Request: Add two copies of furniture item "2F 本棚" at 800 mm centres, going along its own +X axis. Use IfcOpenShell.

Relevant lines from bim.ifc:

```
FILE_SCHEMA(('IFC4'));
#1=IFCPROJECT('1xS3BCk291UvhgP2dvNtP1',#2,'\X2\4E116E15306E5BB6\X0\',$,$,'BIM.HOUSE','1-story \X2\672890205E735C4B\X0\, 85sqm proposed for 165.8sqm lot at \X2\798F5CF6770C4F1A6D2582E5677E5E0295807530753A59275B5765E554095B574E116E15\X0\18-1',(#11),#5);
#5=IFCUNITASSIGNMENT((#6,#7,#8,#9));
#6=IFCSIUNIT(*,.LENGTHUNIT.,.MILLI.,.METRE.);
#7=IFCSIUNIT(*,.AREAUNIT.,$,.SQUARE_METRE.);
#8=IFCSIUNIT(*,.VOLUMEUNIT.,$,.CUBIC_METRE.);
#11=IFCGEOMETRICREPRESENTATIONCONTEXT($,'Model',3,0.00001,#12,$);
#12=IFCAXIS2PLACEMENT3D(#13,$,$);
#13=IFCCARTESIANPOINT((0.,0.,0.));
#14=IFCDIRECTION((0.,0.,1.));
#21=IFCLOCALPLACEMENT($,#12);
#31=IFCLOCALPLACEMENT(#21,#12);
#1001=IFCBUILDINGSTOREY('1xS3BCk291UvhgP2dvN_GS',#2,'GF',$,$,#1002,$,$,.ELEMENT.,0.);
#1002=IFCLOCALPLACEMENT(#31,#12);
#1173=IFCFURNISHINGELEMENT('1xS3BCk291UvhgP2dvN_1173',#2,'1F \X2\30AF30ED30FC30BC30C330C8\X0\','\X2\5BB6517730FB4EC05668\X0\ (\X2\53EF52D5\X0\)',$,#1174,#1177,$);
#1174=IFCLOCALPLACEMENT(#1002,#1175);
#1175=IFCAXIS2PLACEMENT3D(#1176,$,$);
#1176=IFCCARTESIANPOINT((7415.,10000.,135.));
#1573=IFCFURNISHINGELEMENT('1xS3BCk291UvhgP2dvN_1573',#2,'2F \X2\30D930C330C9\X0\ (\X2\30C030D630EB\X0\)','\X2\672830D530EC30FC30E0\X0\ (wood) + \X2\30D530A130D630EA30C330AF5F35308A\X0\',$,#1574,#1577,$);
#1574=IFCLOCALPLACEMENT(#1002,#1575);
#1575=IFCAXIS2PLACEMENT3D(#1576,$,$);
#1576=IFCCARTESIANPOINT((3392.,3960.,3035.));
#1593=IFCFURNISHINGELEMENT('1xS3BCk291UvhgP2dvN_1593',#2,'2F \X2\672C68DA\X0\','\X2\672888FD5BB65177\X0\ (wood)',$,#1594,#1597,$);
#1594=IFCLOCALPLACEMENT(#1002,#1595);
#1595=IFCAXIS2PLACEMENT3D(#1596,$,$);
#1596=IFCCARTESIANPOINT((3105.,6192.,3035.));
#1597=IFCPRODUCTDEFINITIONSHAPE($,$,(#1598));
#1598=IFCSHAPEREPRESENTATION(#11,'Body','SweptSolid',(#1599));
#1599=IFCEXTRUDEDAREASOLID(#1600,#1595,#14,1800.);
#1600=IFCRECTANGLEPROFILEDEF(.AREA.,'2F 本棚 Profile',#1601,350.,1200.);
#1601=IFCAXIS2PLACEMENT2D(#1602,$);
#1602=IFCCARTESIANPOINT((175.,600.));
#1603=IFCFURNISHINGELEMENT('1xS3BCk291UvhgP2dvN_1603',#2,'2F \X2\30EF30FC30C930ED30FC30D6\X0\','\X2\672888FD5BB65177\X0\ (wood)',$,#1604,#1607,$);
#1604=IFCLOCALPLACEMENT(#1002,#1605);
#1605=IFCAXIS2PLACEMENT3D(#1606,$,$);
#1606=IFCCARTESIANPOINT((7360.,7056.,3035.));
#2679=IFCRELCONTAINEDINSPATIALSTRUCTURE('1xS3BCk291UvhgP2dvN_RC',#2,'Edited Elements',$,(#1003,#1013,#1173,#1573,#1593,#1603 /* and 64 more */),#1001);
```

```python
import ifcopenshell
import ifcopenshell.api.geometry
import ifcopenshell.api.root
import ifcopenshell.util.element
import ifcopenshell.util.placement
import ifcopenshell.util.unit

model = ifcopenshell.open("bim.ifc")
unit_scale = ifcopenshell.util.unit.calculate_unit_scale(model)


def reuse_history(source, copy):
    """copy_class also copies each property set's owner history, people and application; keep the originals."""
    for rel in copy.IsDefinedBy:
        if rel.is_a("IfcRelDefinesByProperties") and (history := rel.RelatingPropertyDefinition.OwnerHistory):
            rel.RelatingPropertyDefinition.OwnerHistory = source.OwnerHistory
            ifcopenshell.util.element.remove_deep2(model, history)


source = model.by_id(1593)
base = ifcopenshell.util.placement.get_local_placement(source.ObjectPlacement)
step = base[:3, 0] * 0.8 / unit_scale

for i in range(1, 3):
    copy = ifcopenshell.api.root.copy_class(model, product=source)
    copy.Representation = ifcopenshell.util.element.copy_deep(
        model, source.Representation, exclude=["IfcGeometricRepresentationContext", "IfcRepresentationMap"]
    )
    reuse_history(source, copy)
    matrix = base.copy()
    matrix[:3, 3] += i * step
    print("added at", matrix[:3, 3].round(3) + 0.0)
    ifcopenshell.api.geometry.edit_object_placement(model, product=copy, matrix=matrix, is_si=False)

model.write("bim-out.ifc")
```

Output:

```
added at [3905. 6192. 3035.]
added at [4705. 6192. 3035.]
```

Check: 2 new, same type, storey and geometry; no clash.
